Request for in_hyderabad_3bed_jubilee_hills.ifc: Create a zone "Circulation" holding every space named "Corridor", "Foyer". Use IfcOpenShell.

First a look at what the model holds.

```python
import ifcopenshell

model = ifcopenshell.open("in_hyderabad_3bed_jubilee_hills.ifc")
print(model.schema)
seen = {}
for space in model.by_type("IfcSpace"):
    seen[space.LongName] = seen.get(space.LongName, 0) + 1
for name, count in sorted(seen.items(), key=str):
    print(count, "x", name)
print("zones:", [z.Name for z in model.by_type("IfcZone")][:20])
```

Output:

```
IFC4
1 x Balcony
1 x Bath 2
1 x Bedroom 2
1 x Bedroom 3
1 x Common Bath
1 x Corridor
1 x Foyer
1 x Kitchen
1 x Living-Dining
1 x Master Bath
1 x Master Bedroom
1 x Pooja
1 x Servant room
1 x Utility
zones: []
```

```python
import ifcopenshell
import ifcopenshell.api.group
import ifcopenshell.api.root

model = ifcopenshell.open("in_hyderabad_3bed_jubilee_hills.ifc")

names = {"Corridor", "Foyer"}
spaces = [s for s in model.by_type("IfcSpace") if s.LongName in names]

zone = ifcopenshell.api.root.create_entity(model, ifc_class="IfcZone", name="Circulation")
ifcopenshell.api.group.assign_group(model, products=spaces, group=zone)
print(len(spaces), "spaces in", zone.Name)

model.write("in_hyderabad_3bed_jubilee_hills_edited.ifc")
```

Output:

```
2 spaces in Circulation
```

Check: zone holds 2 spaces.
